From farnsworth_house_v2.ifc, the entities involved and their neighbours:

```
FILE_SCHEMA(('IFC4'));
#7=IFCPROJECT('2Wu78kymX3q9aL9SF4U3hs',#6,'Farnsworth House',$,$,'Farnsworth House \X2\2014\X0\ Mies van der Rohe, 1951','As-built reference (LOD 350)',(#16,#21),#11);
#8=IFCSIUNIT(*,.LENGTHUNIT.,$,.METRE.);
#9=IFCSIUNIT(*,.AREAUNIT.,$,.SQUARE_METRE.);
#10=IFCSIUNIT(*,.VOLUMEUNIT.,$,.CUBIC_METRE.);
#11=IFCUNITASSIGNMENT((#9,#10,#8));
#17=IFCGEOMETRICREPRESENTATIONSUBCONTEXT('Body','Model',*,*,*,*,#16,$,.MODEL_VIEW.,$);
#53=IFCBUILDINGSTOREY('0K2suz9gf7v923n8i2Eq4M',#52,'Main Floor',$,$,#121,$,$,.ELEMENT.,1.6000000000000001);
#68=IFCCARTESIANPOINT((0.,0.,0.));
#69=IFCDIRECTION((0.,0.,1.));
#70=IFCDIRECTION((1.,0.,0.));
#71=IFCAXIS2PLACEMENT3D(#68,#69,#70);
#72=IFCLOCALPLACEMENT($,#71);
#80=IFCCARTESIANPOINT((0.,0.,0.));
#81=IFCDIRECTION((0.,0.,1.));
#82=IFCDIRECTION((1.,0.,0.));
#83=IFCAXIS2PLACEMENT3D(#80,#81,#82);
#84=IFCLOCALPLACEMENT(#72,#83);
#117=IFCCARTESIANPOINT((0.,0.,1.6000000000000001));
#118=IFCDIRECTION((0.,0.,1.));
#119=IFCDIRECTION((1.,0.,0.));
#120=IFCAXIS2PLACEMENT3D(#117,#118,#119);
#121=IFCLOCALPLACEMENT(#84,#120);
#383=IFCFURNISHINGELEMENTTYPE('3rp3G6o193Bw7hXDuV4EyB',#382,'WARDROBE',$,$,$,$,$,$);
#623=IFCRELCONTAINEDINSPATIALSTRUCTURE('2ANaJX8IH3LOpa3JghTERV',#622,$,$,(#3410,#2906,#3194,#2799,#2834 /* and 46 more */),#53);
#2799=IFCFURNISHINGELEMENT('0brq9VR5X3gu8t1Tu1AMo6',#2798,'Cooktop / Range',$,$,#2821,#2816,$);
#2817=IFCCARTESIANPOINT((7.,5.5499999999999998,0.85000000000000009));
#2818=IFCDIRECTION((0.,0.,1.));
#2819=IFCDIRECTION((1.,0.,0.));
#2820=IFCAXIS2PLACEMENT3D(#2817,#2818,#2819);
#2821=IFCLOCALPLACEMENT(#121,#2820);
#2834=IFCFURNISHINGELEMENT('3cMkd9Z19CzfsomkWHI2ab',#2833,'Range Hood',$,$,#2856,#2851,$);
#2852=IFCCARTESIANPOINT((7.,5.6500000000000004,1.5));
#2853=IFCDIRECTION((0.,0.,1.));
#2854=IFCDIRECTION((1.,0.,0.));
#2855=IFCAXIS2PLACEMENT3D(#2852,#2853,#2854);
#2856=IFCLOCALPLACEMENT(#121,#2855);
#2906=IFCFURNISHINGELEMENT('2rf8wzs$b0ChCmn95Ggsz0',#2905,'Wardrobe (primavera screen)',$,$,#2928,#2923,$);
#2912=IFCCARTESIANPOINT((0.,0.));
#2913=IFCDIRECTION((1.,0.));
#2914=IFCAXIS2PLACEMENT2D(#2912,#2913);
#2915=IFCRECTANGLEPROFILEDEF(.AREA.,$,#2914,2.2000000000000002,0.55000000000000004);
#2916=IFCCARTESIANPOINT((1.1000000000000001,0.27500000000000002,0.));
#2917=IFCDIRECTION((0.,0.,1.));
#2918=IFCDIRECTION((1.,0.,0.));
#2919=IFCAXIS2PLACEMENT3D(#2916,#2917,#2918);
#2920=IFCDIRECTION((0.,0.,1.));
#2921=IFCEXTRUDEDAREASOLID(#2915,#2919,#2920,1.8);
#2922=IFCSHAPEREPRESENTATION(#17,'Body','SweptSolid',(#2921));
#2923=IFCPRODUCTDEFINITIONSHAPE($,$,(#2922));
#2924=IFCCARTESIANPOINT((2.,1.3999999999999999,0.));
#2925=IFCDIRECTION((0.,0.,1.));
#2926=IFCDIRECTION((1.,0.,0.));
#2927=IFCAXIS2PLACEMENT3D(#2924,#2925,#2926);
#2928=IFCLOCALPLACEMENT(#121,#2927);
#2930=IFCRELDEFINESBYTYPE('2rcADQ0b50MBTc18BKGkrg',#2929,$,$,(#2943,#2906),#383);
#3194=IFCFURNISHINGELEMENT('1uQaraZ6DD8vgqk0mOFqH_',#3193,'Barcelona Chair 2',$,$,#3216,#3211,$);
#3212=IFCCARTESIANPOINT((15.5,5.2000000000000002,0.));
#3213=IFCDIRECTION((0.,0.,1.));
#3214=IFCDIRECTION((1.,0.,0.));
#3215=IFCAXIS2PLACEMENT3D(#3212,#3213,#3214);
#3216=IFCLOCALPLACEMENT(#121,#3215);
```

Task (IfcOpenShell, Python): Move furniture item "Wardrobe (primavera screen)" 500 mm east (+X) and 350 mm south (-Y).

```python
import ifcopenshell
import ifcopenshell.api.geometry
import ifcopenshell.util.placement
import ifcopenshell.util.unit

model = ifcopenshell.open("farnsworth_house_v2.ifc")
unit_scale = ifcopenshell.util.unit.calculate_unit_scale(model)

item = model.by_guid("2rf8wzs$b0ChCmn95Ggsz0")
matrix = ifcopenshell.util.placement.get_local_placement(item.ObjectPlacement)
matrix[0, 3] += 0.5 / unit_scale
matrix[1, 3] -= 0.35 / unit_scale
ifcopenshell.api.geometry.edit_object_placement(model, product=item, matrix=matrix, is_si=False)

print(ifcopenshell.util.placement.get_local_placement(item.ObjectPlacement).round(3) + 0.0)

model.write("farnsworth_house_v2_rev.ifc")
```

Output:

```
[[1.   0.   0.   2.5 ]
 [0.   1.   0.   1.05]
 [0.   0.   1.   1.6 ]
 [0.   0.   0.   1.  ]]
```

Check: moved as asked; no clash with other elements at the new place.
